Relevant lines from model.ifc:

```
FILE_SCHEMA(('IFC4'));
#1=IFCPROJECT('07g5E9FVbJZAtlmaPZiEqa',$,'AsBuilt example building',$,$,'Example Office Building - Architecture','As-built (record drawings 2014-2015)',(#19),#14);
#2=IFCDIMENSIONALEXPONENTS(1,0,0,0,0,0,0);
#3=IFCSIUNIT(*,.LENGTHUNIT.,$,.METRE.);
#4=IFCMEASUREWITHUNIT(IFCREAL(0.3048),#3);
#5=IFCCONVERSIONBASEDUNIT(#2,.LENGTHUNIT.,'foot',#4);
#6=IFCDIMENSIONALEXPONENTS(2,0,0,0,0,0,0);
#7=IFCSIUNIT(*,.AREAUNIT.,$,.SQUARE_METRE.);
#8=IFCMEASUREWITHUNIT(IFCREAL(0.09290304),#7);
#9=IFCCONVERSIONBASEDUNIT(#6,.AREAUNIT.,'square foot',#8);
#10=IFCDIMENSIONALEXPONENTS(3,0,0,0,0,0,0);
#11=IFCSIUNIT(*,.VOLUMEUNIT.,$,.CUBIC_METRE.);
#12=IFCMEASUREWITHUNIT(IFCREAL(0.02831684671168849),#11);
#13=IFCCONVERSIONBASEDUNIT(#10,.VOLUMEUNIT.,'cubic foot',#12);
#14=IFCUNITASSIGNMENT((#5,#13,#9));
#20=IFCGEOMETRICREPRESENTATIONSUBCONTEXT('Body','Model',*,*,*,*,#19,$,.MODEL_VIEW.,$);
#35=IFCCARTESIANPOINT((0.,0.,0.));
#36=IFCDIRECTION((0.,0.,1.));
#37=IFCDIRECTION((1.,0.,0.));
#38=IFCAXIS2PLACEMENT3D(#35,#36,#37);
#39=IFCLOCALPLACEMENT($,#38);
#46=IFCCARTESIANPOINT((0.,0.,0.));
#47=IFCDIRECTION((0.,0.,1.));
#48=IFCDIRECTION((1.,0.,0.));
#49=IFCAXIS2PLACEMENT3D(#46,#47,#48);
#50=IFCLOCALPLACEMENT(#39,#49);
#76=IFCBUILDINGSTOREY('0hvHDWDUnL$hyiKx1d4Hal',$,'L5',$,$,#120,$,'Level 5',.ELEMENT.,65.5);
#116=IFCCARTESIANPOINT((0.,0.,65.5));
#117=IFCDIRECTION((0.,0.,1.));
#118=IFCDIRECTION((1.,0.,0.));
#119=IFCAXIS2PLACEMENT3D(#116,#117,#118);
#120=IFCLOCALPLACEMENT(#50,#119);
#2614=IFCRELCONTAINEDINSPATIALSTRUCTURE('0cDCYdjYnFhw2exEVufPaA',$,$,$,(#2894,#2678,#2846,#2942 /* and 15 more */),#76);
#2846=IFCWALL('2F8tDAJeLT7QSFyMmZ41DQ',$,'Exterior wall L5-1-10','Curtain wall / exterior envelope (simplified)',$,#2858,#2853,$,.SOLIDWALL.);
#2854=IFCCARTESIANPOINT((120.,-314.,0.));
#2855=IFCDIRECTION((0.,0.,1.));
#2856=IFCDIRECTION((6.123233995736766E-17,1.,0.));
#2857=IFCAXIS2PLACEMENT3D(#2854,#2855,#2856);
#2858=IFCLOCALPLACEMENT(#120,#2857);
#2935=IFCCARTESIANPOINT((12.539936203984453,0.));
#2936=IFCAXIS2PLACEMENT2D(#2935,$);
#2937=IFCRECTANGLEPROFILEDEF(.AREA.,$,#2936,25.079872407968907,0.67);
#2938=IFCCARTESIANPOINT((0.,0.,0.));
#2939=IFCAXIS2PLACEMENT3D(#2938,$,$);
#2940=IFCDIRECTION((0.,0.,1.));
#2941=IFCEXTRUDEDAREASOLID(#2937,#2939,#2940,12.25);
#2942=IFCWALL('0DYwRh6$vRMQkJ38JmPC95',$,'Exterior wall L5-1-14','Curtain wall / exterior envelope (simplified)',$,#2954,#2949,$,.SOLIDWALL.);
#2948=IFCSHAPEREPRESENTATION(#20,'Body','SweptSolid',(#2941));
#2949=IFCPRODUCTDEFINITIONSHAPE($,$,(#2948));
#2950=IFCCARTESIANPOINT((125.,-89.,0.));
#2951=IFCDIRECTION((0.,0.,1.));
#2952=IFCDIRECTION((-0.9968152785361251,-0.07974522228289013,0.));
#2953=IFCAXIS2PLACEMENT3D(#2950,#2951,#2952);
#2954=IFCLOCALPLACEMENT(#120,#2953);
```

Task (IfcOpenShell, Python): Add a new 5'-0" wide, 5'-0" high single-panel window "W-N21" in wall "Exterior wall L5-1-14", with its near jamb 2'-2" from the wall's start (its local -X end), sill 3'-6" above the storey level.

```python
import numpy as np
import ifcopenshell
import ifcopenshell.api.feature
import ifcopenshell.api.geometry
import ifcopenshell.api.root
import ifcopenshell.api.spatial
import ifcopenshell.geom
import ifcopenshell.util.element
import ifcopenshell.util.placement
import ifcopenshell.util.representation
import ifcopenshell.util.shape
import ifcopenshell.util.unit

model = ifcopenshell.open("model.ifc")
unit_scale = ifcopenshell.util.unit.calculate_unit_scale(model)
settings = ifcopenshell.geom.settings()


def volume(element):
    """Net volume in cubic metres, openings subtracted."""
    shape = ifcopenshell.geom.create_shape(settings, element)
    return ifcopenshell.util.shape.get_volume(shape.geometry)


wall = model.by_guid("0DYwRh6$vRMQkJ38JmPC95")
storey = ifcopenshell.util.element.get_container(wall, ifc_class="IfcBuildingStorey")
context = ifcopenshell.util.representation.get_context(model, "Model", "Body", "MODEL_VIEW")
before = volume(wall)

width, height, from_end, sill = 1.524, 1.524, 0.6604, 1.0668  # metres

# The wall runs along its own X axis, and the end named is its -X end.
wall_shape = ifcopenshell.geom.create_shape(settings, wall)
x, y, z = ifcopenshell.util.shape.get_vertices(wall_shape.geometry).T
start = x.min() + from_end
face, thickness = float(y.min()), float(y.max() - y.min())
wall_matrix = ifcopenshell.util.placement.get_local_placement(wall.ObjectPlacement)
level = ifcopenshell.util.placement.get_local_placement(storey.ObjectPlacement)[2, 3]


def in_wall(x, y):
    """Placement at x, y metres in the wall's axes, at sill height."""
    matrix = wall_matrix.copy()
    matrix[:, 3] = wall_matrix @ np.array([x / unit_scale, y / unit_scale, 0.0, 1.0])
    matrix[2, 3] = level + sill / unit_scale
    return matrix


# Opening: a box that overshoots both wall faces by 50 mm.
opening = ifcopenshell.api.root.create_entity(model, ifc_class="IfcOpeningElement", predefined_type="OPENING")
box = ifcopenshell.api.geometry.add_wall_representation(
    model, context=context, length=width, height=height, thickness=thickness + 0.1
)
ifcopenshell.api.geometry.assign_representation(model, product=opening, representation=box)
ifcopenshell.api.geometry.edit_object_placement(model, product=opening, matrix=in_wall(start, face - 0.05), is_si=False)
ifcopenshell.api.feature.add_feature(model, feature=opening, element=wall)

window = ifcopenshell.api.root.create_entity(model, ifc_class="IfcWindow", name="W-N21", predefined_type="WINDOW")
window.OverallWidth, window.OverallHeight = width / unit_scale, height / unit_scale
window.PartitioningType = "SINGLE_PANEL"
body = ifcopenshell.api.geometry.add_window_representation(
    model,
    context=context,
    overall_width=window.OverallWidth,
    overall_height=window.OverallHeight,
    partition_type="SINGLE_PANEL",
)
ifcopenshell.api.geometry.assign_representation(model, product=window, representation=body)
ifcopenshell.api.spatial.assign_container(model, products=[window], relating_structure=storey)
ifcopenshell.api.feature.add_filling(model, opening=opening, element=window)

# Centre the window in the wall's thickness.
ifcopenshell.api.geometry.edit_object_placement(model, product=window, matrix=in_wall(start, face), is_si=False)
window_shape = ifcopenshell.geom.create_shape(settings, window)
depth = ifcopenshell.util.shape.get_vertices(window_shape.geometry)[:, 1]
offset = face + thickness / 2 - (depth.min() + depth.max()) / 2
ifcopenshell.api.geometry.edit_object_placement(model, product=window, matrix=in_wall(start, offset), is_si=False)

after = volume(wall)

print(f"wall volume {before:.3f} -> {after:.3f} m3")

model.write("model_v2.ifc")
```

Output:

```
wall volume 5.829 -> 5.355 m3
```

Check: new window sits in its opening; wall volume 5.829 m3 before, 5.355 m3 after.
